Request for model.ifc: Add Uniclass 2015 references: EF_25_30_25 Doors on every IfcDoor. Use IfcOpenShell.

First a look at what the model holds.

```python
import ifcopenshell

model = ifcopenshell.open("model.ifc")
print(model.schema)
print("classifications:", [c.Name for c in model.by_type("IfcClassification")])
for ifc_class in ("IfcDoor", "IfcRoof", "IfcStair", "IfcWall", "IfcWindow"):
    print(ifc_class, len(model.by_type(ifc_class)))
```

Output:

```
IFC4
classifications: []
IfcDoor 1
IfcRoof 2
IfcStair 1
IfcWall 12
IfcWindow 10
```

```python
import ifcopenshell
import ifcopenshell.api.classification

model = ifcopenshell.open("model.ifc")

system = ifcopenshell.api.classification.add_classification(model, classification="Uniclass 2015")

codes = {
    "IfcDoor": ("EF_25_30_25", "Doors"),
}
for ifc_class, (code, name) in codes.items():
    products = model.by_type(ifc_class)
    ifcopenshell.api.classification.add_reference(
        model, products=products, classification=system, identification=code, name=name
    )
    print(code, len(products))

model.write("model-out.ifc")
```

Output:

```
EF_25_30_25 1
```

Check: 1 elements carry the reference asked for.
